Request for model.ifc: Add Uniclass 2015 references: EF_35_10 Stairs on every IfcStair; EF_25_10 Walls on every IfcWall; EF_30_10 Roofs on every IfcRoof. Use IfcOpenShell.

First a look at what the model holds.

```python
import ifcopenshell

model = ifcopenshell.open("model.ifc")
print(model.schema)
print("classifications:", [c.Name for c in model.by_type("IfcClassification")])
for ifc_class in ("IfcDoor", "IfcRoof", "IfcStair", "IfcWall", "IfcWindow"):
    print(ifc_class, len(model.by_type(ifc_class)))
```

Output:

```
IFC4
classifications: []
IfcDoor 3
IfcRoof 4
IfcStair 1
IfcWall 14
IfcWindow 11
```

```python
import ifcopenshell
import ifcopenshell.api.classification

model = ifcopenshell.open("model.ifc")

system = ifcopenshell.api.classification.add_classification(model, classification="Uniclass 2015")

codes = {
    "IfcStair": ("EF_35_10", "Stairs"),
    "IfcWall": ("EF_25_10", "Walls"),
    "IfcRoof": ("EF_30_10", "Roofs"),
}
for ifc_class, (code, name) in codes.items():
    products = model.by_type(ifc_class)
    ifcopenshell.api.classification.add_reference(
        model, products=products, classification=system, identification=code, name=name
    )
    print(code, len(products))

model.write("model_v2.ifc")
```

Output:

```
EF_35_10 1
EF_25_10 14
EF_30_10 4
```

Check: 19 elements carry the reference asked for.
